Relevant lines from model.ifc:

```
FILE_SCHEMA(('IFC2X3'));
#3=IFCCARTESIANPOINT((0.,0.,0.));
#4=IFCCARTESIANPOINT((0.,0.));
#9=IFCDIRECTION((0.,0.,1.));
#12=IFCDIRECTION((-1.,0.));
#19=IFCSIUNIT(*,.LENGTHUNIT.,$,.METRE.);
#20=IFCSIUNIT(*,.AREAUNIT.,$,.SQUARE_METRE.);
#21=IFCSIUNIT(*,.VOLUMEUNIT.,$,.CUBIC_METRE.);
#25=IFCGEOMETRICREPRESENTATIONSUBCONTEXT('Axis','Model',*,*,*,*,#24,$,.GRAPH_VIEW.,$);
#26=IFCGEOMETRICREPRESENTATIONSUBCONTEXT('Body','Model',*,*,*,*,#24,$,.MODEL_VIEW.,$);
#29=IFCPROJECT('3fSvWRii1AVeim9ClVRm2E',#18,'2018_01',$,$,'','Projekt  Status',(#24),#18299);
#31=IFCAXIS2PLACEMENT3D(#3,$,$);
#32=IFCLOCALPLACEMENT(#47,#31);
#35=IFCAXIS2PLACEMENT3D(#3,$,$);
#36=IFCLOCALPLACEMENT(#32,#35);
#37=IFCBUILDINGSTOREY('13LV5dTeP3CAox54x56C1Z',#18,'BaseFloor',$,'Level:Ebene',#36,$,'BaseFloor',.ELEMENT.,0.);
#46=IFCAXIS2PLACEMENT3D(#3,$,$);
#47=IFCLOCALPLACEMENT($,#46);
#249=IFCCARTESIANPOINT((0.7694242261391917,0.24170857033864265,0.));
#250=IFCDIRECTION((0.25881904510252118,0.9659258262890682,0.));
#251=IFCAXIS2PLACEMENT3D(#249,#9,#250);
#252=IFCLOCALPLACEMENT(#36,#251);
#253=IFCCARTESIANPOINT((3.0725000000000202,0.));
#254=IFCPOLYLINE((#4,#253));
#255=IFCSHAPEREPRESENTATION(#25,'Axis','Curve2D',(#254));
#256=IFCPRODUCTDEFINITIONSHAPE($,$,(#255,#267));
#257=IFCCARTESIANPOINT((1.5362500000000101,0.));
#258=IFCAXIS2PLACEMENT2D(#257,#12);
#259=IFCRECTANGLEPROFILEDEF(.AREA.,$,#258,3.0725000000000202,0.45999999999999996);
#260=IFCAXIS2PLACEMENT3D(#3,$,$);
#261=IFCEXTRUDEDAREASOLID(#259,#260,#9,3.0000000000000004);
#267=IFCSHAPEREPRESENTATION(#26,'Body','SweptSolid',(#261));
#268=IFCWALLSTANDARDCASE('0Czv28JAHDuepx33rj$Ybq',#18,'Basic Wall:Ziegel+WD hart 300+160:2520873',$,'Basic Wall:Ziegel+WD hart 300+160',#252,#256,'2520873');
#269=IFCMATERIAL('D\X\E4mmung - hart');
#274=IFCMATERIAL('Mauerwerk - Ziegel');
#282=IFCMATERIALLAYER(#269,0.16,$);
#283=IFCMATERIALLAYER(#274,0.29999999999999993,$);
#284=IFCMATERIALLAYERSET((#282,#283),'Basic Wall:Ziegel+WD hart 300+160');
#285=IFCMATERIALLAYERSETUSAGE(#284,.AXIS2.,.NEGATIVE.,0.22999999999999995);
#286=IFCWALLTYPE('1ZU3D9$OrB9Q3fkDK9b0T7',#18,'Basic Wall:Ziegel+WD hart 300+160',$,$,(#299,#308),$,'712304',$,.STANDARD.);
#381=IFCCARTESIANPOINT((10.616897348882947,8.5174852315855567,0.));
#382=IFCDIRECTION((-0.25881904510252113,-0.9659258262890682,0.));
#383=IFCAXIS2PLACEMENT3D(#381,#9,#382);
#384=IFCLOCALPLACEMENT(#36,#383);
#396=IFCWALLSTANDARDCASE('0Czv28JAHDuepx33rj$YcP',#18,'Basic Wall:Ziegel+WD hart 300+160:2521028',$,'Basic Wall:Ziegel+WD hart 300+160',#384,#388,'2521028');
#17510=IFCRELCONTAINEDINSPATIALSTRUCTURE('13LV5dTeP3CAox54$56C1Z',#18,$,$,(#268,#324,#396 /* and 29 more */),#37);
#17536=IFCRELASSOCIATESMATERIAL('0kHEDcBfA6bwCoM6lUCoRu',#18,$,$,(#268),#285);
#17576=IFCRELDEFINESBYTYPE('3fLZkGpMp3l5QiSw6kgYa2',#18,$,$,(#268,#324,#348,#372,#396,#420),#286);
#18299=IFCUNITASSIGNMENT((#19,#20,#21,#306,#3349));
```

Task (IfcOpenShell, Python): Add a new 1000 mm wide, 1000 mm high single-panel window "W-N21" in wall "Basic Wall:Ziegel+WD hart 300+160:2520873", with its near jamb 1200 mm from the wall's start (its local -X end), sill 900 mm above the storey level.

```python
import numpy as np
import ifcopenshell
import ifcopenshell.api.feature
import ifcopenshell.api.geometry
import ifcopenshell.api.root
import ifcopenshell.api.spatial
import ifcopenshell.api.type
import ifcopenshell.geom
import ifcopenshell.util.element
import ifcopenshell.util.placement
import ifcopenshell.util.representation
import ifcopenshell.util.shape
import ifcopenshell.util.unit

model = ifcopenshell.open("model.ifc")
unit_scale = ifcopenshell.util.unit.calculate_unit_scale(model)
settings = ifcopenshell.geom.settings()


def volume(element):
    """Net volume in cubic metres, openings subtracted."""
    shape = ifcopenshell.geom.create_shape(settings, element)
    return ifcopenshell.util.shape.get_volume(shape.geometry)


wall = model.by_guid("0Czv28JAHDuepx33rj$Ybq")
storey = ifcopenshell.util.element.get_container(wall, ifc_class="IfcBuildingStorey")
context = ifcopenshell.util.representation.get_context(model, "Model", "Body", "MODEL_VIEW")
before = volume(wall)

width, height, from_end, sill = 1, 1, 1.2, 0.9  # metres

# The wall runs along its own X axis, and the end named is its -X end.
wall_shape = ifcopenshell.geom.create_shape(settings, wall)
x, y, z = ifcopenshell.util.shape.get_vertices(wall_shape.geometry).T
start = x.min() + from_end
face, thickness = float(y.min()), float(y.max() - y.min())
wall_matrix = ifcopenshell.util.placement.get_local_placement(wall.ObjectPlacement)
level = ifcopenshell.util.placement.get_local_placement(storey.ObjectPlacement)[2, 3]


def in_wall(x, y):
    """Placement at x, y metres in the wall's axes, at sill height."""
    matrix = wall_matrix.copy()
    matrix[:, 3] = wall_matrix @ np.array([x / unit_scale, y / unit_scale, 0.0, 1.0])
    matrix[2, 3] = level + sill / unit_scale
    return matrix


# Opening: a box that overshoots both wall faces by 50 mm.
opening = ifcopenshell.api.root.create_entity(model, ifc_class="IfcOpeningElement")
box = ifcopenshell.api.geometry.add_wall_representation(
    model, context=context, length=width, height=height, thickness=thickness + 0.1
)
ifcopenshell.api.geometry.assign_representation(model, product=opening, representation=box)
ifcopenshell.api.geometry.edit_object_placement(model, product=opening, matrix=in_wall(start, face - 0.05), is_si=False)
ifcopenshell.api.feature.add_feature(model, feature=opening, element=wall)

window = ifcopenshell.api.root.create_entity(model, ifc_class="IfcWindow", name="W-N21")
window.OverallWidth, window.OverallHeight = width / unit_scale, height / unit_scale
body = ifcopenshell.api.geometry.add_window_representation(
    model,
    context=context,
    overall_width=window.OverallWidth,
    overall_height=window.OverallHeight,
    partition_type="SINGLE_PANEL",
)
ifcopenshell.api.geometry.assign_representation(model, product=window, representation=body)
ifcopenshell.api.spatial.assign_container(model, products=[window], relating_structure=storey)
fills = ifcopenshell.api.feature.add_filling(model, opening=opening, element=window)
fills.OwnerHistory = window.OwnerHistory  # required in IFC2X3

# IFC2X3 keeps the operation on the window style.
style = ifcopenshell.api.root.create_entity(model, ifc_class="IfcWindowStyle", name="W-N21")
style.OperationType, style.ConstructionType = "SINGLE_PANEL", "NOTDEFINED"
style.ParameterTakesPrecedence = style.Sizeable = False
ifcopenshell.api.type.assign_type(model, related_objects=[window], relating_type=style)

# Centre the window in the wall's thickness.
ifcopenshell.api.geometry.edit_object_placement(model, product=window, matrix=in_wall(start, face), is_si=False)
window_shape = ifcopenshell.geom.create_shape(settings, window)
depth = ifcopenshell.util.shape.get_vertices(window_shape.geometry)[:, 1]
offset = face + thickness / 2 - (depth.min() + depth.max()) / 2
ifcopenshell.api.geometry.edit_object_placement(model, product=window, matrix=in_wall(start, offset), is_si=False)

after = volume(wall)

print(f"wall volume {before:.3f} -> {after:.3f} m3")

model.write("model_updated.ifc")
```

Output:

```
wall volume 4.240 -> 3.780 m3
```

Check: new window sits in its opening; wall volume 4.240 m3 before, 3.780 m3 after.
